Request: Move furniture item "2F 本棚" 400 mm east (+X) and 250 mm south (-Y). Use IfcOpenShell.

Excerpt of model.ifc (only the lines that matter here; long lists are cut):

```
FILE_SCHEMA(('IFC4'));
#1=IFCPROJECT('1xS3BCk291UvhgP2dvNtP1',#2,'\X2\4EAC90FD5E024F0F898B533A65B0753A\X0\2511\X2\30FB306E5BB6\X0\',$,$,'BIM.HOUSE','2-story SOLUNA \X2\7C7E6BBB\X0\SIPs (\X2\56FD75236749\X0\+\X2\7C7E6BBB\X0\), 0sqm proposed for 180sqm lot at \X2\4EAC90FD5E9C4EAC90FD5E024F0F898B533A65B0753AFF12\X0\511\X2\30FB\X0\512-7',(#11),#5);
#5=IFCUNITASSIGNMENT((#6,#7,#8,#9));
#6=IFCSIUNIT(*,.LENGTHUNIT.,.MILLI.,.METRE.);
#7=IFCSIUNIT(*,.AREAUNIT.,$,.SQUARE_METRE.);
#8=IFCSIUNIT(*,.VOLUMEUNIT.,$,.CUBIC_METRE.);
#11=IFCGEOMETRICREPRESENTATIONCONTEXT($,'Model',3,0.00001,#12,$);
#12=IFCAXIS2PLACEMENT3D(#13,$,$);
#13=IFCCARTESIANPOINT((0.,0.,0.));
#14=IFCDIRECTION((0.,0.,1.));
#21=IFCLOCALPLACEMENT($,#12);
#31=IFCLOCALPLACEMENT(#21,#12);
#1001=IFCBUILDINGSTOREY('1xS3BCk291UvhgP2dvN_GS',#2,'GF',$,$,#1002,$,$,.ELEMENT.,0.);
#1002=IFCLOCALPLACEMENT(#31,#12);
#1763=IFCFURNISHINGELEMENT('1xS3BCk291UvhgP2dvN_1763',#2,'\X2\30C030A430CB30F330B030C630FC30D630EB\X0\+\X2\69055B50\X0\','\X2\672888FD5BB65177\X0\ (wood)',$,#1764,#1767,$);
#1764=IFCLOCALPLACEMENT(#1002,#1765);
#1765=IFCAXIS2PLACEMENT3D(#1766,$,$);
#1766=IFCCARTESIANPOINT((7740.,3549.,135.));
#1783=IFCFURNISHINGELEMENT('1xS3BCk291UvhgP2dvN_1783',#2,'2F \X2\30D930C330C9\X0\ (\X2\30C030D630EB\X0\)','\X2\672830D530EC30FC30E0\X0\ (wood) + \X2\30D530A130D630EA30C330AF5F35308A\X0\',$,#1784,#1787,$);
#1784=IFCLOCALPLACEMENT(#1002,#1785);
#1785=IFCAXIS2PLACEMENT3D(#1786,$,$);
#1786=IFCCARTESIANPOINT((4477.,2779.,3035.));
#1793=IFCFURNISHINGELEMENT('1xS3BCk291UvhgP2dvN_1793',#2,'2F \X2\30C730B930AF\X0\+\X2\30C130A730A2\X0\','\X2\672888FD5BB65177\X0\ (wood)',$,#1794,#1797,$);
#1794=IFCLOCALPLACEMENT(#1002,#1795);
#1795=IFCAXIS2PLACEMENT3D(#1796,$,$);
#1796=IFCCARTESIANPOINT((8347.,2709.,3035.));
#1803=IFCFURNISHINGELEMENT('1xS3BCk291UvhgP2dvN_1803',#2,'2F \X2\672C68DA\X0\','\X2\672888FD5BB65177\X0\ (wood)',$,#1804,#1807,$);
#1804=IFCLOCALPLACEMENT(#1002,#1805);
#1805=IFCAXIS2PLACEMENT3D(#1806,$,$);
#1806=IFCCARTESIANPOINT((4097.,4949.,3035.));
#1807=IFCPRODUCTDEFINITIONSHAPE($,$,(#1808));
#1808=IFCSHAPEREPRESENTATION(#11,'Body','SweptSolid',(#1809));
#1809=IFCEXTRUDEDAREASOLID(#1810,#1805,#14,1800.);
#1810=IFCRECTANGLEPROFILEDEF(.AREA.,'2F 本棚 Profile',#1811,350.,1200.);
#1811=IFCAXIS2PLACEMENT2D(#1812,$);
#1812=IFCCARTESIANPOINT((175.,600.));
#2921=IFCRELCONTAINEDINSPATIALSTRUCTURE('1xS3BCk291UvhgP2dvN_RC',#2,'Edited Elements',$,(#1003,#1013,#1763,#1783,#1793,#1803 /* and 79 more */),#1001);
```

```python
import ifcopenshell
import ifcopenshell.api.geometry
import ifcopenshell.util.placement
import ifcopenshell.util.unit

model = ifcopenshell.open("model.ifc")
unit_scale = ifcopenshell.util.unit.calculate_unit_scale(model)

item = model.by_guid("1xS3BCk291UvhgP2dvN_1803")
matrix = ifcopenshell.util.placement.get_local_placement(item.ObjectPlacement)
matrix[0, 3] += 0.4 / unit_scale
matrix[1, 3] -= 0.25 / unit_scale
ifcopenshell.api.geometry.edit_object_placement(model, product=item, matrix=matrix, is_si=False)

print(ifcopenshell.util.placement.get_local_placement(item.ObjectPlacement).round(3) + 0.0)

model.write("model_updated.ifc")
```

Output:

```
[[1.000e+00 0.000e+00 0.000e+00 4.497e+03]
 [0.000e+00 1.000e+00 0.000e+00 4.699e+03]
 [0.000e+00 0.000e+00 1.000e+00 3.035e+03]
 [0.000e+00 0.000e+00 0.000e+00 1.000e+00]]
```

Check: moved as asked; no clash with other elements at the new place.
